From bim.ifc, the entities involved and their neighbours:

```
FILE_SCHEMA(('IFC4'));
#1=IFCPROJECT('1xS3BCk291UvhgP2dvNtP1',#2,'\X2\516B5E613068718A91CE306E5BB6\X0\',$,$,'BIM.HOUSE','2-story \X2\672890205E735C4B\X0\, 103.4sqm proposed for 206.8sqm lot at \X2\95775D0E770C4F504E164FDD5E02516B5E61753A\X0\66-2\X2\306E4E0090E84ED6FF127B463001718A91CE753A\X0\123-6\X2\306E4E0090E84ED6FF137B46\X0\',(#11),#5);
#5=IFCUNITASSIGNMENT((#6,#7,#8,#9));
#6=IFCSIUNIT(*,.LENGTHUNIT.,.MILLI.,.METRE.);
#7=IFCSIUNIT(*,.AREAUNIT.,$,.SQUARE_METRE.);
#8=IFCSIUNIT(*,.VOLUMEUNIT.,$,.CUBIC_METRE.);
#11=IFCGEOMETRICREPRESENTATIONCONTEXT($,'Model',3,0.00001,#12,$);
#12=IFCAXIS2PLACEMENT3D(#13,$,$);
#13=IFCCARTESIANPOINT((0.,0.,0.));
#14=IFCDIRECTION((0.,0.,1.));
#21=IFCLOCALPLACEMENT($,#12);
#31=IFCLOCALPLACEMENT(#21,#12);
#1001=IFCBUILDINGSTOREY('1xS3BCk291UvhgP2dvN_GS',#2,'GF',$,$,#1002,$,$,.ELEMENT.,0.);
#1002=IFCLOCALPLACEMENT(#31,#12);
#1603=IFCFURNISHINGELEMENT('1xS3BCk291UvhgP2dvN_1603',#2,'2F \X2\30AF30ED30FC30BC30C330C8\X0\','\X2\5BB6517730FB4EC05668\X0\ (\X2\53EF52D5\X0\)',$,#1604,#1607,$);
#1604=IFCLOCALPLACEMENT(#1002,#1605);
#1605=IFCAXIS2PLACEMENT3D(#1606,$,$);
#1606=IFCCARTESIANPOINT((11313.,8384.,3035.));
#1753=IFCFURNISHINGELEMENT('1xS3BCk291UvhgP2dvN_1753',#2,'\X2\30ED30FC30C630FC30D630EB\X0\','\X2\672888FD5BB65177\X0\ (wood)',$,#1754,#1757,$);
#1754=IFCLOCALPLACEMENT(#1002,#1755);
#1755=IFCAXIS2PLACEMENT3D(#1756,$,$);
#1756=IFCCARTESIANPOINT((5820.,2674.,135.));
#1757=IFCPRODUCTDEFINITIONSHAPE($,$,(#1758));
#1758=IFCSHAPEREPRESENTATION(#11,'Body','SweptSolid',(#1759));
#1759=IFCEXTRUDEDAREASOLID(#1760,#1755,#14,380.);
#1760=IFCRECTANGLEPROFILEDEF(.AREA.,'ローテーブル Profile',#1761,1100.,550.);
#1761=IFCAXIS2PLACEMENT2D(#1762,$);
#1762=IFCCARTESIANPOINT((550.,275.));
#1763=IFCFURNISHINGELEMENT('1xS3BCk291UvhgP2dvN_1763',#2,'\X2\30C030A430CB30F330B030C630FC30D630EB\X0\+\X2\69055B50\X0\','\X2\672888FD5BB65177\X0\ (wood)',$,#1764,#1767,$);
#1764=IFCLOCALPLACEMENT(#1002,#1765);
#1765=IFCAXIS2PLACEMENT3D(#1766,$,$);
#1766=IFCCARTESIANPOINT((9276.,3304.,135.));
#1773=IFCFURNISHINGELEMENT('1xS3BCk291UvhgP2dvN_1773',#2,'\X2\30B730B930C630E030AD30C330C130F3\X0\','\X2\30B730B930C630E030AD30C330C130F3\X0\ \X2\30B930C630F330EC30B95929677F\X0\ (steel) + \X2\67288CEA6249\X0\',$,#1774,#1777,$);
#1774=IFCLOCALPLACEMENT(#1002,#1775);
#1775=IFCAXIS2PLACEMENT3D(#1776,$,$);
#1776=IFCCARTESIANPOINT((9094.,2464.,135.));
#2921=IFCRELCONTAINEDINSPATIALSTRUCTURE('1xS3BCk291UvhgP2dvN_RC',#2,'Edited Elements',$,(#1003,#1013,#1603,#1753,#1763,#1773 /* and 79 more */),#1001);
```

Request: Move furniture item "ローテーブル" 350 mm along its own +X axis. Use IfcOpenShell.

```python
import ifcopenshell
import ifcopenshell.api.geometry
import ifcopenshell.util.placement
import ifcopenshell.util.unit

model = ifcopenshell.open("bim.ifc")
unit_scale = ifcopenshell.util.unit.calculate_unit_scale(model)

item = model.by_guid("1xS3BCk291UvhgP2dvN_1753")
matrix = ifcopenshell.util.placement.get_local_placement(item.ObjectPlacement)
matrix[:3, 3] += matrix[:3, 0] * 0.35 / unit_scale
ifcopenshell.api.geometry.edit_object_placement(model, product=item, matrix=matrix, is_si=False)

print(ifcopenshell.util.placement.get_local_placement(item.ObjectPlacement).round(3) + 0.0)

model.write("bim_updated.ifc")
```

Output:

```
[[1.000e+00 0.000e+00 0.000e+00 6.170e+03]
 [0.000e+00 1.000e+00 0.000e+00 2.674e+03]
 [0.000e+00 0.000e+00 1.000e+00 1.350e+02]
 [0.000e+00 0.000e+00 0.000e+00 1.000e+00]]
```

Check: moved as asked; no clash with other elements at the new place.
